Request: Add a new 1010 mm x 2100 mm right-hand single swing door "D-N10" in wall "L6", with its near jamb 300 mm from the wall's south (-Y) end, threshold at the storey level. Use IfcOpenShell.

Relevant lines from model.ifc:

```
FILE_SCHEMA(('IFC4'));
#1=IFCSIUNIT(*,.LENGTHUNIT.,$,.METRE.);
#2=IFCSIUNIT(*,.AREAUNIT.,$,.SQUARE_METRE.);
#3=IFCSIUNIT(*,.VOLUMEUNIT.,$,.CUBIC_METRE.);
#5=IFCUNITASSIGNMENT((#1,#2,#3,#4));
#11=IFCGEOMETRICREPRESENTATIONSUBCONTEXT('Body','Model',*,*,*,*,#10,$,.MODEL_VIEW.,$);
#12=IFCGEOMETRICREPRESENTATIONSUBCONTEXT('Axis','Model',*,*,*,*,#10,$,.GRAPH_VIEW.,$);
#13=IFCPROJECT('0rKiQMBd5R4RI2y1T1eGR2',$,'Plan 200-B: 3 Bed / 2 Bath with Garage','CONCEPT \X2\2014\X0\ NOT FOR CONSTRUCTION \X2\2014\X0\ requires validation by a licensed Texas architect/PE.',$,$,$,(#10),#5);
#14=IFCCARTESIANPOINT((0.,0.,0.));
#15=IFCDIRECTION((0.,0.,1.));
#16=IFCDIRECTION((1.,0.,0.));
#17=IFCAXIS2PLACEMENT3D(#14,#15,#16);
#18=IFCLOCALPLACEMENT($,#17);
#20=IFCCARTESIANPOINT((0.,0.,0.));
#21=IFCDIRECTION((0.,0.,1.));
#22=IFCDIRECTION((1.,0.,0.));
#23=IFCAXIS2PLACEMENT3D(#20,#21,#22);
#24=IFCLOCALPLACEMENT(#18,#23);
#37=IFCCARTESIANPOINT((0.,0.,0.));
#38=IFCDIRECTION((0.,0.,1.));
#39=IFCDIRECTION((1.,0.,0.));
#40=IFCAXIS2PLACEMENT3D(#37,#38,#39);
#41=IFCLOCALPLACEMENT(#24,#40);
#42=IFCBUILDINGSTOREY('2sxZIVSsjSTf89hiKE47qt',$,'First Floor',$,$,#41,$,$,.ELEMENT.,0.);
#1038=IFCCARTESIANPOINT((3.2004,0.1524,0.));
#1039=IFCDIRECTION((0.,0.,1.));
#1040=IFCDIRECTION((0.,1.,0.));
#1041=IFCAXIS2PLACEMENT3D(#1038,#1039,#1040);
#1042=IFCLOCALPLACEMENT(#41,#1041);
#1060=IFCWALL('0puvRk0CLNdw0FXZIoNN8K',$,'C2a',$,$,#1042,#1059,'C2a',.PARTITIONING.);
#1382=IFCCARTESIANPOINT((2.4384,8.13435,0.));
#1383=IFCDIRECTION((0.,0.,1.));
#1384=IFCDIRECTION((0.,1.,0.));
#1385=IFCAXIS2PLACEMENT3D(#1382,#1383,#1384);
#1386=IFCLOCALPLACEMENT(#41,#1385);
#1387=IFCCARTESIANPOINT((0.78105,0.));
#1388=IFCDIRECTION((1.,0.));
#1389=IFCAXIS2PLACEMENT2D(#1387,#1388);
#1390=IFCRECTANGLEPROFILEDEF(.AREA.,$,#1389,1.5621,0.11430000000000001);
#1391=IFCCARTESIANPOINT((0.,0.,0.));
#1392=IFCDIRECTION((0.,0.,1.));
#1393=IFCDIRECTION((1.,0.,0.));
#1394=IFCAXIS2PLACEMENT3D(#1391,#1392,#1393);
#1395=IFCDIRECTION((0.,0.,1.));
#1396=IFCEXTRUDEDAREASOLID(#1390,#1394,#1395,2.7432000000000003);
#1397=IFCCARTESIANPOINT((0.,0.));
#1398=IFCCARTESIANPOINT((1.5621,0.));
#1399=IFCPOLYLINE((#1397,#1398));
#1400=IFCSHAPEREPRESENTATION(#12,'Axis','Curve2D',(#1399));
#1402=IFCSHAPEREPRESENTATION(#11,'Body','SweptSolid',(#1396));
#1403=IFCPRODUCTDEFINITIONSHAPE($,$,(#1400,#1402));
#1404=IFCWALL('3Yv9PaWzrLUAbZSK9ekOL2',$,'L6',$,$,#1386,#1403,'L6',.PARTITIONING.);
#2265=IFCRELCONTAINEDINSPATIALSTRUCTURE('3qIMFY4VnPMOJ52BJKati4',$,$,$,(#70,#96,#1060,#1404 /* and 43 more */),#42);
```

```python
import numpy as np
import ifcopenshell
import ifcopenshell.api.feature
import ifcopenshell.api.geometry
import ifcopenshell.api.root
import ifcopenshell.api.spatial
import ifcopenshell.geom
import ifcopenshell.util.element
import ifcopenshell.util.placement
import ifcopenshell.util.representation
import ifcopenshell.util.shape
import ifcopenshell.util.unit

model = ifcopenshell.open("model.ifc")
unit_scale = ifcopenshell.util.unit.calculate_unit_scale(model)
settings = ifcopenshell.geom.settings()


def volume(element):
    """Net volume in cubic metres, openings subtracted."""
    shape = ifcopenshell.geom.create_shape(settings, element)
    return ifcopenshell.util.shape.get_volume(shape.geometry)


wall = model.by_id(1404)
storey = ifcopenshell.util.element.get_container(wall, ifc_class="IfcBuildingStorey")
context = ifcopenshell.util.representation.get_context(model, "Model", "Body", "MODEL_VIEW")
before = volume(wall)

width, height, from_end, sill = 1.01, 2.1, 0.3, 0.0  # metres

# The wall runs along its own X axis, and the end named is its -X end.
wall_shape = ifcopenshell.geom.create_shape(settings, wall)
x, y, z = ifcopenshell.util.shape.get_vertices(wall_shape.geometry).T
start = x.min() + from_end
face, thickness = float(y.min()), float(y.max() - y.min())
wall_matrix = ifcopenshell.util.placement.get_local_placement(wall.ObjectPlacement)
level = ifcopenshell.util.placement.get_local_placement(storey.ObjectPlacement)[2, 3]


def in_wall(x, y):
    """Placement at x, y metres in the wall's axes, at sill height."""
    matrix = wall_matrix.copy()
    matrix[:, 3] = wall_matrix @ np.array([x / unit_scale, y / unit_scale, 0.0, 1.0])
    matrix[2, 3] = level + sill / unit_scale
    return matrix


# Opening: a box that overshoots both wall faces by 50 mm.
opening = ifcopenshell.api.root.create_entity(model, ifc_class="IfcOpeningElement", predefined_type="OPENING")
box = ifcopenshell.api.geometry.add_wall_representation(
    model, context=context, length=width, height=height, thickness=thickness + 0.1
)
ifcopenshell.api.geometry.assign_representation(model, product=opening, representation=box)
ifcopenshell.api.geometry.edit_object_placement(model, product=opening, matrix=in_wall(start, face - 0.05), is_si=False)
ifcopenshell.api.feature.add_feature(model, feature=opening, element=wall)

door = ifcopenshell.api.root.create_entity(model, ifc_class="IfcDoor", name="D-N10", predefined_type="DOOR")
door.OverallWidth, door.OverallHeight = width / unit_scale, height / unit_scale
door.OperationType = "SINGLE_SWING_RIGHT"
body = ifcopenshell.api.geometry.add_door_representation(
    model,
    context=context,
    overall_width=door.OverallWidth,
    overall_height=door.OverallHeight,
    operation_type="SINGLE_SWING_RIGHT",
    lining_properties={"LiningDepth": thickness / unit_scale, "ThresholdDepth": thickness / unit_scale},
)
ifcopenshell.api.geometry.assign_representation(model, product=door, representation=body)
ifcopenshell.api.spatial.assign_container(model, products=[door], relating_structure=storey)
ifcopenshell.api.feature.add_filling(model, opening=opening, element=door)

# The lining spans the wall, so the door starts at the wall face.
ifcopenshell.api.geometry.edit_object_placement(model, product=door, matrix=in_wall(start, face), is_si=False)

after = volume(wall)

print(f"wall volume {before:.3f} -> {after:.3f} m3")

model.write("model_rev.ifc")
```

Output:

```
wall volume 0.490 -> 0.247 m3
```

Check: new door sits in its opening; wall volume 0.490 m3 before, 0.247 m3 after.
